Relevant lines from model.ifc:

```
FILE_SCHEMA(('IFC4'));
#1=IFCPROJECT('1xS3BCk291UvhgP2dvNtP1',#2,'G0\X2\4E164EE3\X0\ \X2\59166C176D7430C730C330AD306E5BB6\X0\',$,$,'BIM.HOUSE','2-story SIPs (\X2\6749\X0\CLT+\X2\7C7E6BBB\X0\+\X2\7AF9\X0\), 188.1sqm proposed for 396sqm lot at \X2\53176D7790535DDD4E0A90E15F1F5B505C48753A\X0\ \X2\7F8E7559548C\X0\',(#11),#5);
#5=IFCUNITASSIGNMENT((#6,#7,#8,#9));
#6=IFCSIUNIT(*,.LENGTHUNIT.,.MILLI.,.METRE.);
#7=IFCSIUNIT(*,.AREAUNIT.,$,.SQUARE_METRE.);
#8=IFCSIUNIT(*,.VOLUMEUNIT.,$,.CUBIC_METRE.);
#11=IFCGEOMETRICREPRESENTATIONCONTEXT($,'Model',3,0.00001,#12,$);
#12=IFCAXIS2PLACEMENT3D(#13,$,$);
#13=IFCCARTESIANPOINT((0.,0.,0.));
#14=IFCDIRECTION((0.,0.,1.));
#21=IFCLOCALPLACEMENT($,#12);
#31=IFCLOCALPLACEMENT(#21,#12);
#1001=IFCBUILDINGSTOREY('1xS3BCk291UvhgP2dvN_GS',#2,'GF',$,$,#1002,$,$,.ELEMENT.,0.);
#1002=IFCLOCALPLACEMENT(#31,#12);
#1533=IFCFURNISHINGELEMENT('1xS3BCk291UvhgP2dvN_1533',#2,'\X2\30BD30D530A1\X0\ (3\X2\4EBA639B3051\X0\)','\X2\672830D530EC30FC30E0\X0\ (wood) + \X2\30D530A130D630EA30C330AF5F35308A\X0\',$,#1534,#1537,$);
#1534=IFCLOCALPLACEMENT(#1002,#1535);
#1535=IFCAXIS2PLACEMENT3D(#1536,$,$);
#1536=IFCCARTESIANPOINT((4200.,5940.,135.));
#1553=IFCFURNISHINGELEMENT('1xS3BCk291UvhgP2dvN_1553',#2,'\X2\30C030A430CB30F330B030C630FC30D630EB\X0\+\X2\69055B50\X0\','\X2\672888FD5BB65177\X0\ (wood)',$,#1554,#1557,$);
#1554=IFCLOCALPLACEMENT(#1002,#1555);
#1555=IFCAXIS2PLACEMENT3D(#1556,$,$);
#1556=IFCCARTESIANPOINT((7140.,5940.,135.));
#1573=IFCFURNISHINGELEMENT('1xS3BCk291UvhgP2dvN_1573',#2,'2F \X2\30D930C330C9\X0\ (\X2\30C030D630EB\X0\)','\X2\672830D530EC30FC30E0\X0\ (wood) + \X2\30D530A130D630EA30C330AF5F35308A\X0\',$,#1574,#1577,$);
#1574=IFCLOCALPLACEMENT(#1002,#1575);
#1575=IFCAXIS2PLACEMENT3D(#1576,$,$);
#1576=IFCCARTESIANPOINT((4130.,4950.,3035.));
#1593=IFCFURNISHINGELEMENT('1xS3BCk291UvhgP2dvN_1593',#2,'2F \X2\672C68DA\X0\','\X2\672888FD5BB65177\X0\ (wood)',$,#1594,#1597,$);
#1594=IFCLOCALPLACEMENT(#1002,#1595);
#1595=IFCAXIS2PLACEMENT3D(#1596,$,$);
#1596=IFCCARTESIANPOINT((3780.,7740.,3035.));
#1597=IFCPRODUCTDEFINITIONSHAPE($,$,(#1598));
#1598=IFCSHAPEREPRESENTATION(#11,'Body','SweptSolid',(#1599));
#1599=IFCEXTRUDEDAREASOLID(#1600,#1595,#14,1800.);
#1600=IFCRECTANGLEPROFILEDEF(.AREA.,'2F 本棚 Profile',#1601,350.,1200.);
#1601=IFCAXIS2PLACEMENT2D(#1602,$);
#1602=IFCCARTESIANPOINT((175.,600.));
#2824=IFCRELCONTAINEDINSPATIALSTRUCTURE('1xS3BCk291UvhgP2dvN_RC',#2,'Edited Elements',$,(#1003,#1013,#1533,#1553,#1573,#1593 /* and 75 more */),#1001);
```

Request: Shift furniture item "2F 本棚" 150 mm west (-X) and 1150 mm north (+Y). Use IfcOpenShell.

```python
import ifcopenshell
import ifcopenshell.api.geometry
import ifcopenshell.util.placement
import ifcopenshell.util.unit

model = ifcopenshell.open("model.ifc")
unit_scale = ifcopenshell.util.unit.calculate_unit_scale(model)

item = model.by_guid("1xS3BCk291UvhgP2dvN_1593")
matrix = ifcopenshell.util.placement.get_local_placement(item.ObjectPlacement)
matrix[0, 3] -= 0.15 / unit_scale
matrix[1, 3] += 1.15 / unit_scale
ifcopenshell.api.geometry.edit_object_placement(model, product=item, matrix=matrix, is_si=False)

print(ifcopenshell.util.placement.get_local_placement(item.ObjectPlacement).round(3) + 0.0)

model.write("model-out.ifc")
```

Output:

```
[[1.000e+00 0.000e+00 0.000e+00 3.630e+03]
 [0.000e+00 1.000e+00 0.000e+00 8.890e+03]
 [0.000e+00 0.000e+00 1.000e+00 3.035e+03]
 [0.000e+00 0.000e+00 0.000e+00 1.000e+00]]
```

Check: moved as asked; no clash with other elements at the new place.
